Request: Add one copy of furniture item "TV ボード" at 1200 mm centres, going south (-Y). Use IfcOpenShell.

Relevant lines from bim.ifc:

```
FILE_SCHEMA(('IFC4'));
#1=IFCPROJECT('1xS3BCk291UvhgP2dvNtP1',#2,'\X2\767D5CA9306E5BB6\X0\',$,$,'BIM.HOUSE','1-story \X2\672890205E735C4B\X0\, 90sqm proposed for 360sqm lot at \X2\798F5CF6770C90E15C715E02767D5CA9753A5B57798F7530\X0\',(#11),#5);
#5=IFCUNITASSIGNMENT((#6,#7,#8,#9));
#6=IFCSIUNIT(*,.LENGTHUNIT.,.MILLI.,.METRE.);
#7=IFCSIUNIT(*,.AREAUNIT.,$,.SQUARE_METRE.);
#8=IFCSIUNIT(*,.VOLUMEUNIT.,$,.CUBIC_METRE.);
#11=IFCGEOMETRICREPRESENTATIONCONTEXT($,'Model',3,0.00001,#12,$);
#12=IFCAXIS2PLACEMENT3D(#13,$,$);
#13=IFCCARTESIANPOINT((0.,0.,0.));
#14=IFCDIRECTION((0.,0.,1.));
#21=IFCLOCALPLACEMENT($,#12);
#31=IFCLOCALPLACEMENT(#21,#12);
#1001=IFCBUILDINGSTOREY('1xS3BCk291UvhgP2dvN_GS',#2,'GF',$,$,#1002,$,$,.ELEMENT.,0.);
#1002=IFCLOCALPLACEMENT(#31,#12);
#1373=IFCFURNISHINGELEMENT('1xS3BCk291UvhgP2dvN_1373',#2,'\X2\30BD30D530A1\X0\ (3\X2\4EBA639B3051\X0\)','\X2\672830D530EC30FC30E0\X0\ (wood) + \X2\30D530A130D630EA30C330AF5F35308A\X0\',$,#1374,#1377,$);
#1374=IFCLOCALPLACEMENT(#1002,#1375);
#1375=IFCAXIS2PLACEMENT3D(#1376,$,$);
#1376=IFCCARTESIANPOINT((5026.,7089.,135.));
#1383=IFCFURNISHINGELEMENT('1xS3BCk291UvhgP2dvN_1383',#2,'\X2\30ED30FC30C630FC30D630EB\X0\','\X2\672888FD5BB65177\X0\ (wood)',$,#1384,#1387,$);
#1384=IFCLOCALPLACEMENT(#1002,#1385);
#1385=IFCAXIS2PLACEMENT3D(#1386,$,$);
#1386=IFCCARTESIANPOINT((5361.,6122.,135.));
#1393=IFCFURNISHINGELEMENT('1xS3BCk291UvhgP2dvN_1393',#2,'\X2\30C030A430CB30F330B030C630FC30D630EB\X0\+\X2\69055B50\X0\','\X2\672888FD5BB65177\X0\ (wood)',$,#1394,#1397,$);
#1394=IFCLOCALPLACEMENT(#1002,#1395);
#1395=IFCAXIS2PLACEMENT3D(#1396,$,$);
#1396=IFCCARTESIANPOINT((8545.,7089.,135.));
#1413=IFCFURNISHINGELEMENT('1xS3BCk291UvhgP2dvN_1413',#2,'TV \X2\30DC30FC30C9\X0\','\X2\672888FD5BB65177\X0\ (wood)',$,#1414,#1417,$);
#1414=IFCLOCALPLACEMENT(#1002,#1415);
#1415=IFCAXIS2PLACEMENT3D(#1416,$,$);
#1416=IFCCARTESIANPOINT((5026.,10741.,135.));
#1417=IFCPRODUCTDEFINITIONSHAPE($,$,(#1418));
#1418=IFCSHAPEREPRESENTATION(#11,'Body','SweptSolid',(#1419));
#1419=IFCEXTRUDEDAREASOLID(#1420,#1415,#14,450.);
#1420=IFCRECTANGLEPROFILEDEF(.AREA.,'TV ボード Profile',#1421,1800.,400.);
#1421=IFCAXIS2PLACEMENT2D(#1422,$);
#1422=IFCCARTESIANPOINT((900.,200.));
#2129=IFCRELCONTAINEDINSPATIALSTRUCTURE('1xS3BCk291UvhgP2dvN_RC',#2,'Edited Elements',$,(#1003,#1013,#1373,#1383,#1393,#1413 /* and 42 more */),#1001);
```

```python
import numpy as np
import ifcopenshell
import ifcopenshell.api.geometry
import ifcopenshell.api.root
import ifcopenshell.util.element
import ifcopenshell.util.placement
import ifcopenshell.util.unit

model = ifcopenshell.open("bim.ifc")
unit_scale = ifcopenshell.util.unit.calculate_unit_scale(model)


def reuse_history(source, copy):
    """copy_class also copies each property set's owner history, people and application; keep the originals."""
    for rel in copy.IsDefinedBy:
        if rel.is_a("IfcRelDefinesByProperties") and (history := rel.RelatingPropertyDefinition.OwnerHistory):
            rel.RelatingPropertyDefinition.OwnerHistory = source.OwnerHistory
            ifcopenshell.util.element.remove_deep2(model, history)


source = model.by_id(1413)
base = ifcopenshell.util.placement.get_local_placement(source.ObjectPlacement)
step = np.array([0.0, -1.0, 0.0]) * 1.2 / unit_scale

for i in range(1, 2):
    copy = ifcopenshell.api.root.copy_class(model, product=source)
    copy.Representation = ifcopenshell.util.element.copy_deep(
        model, source.Representation, exclude=["IfcGeometricRepresentationContext", "IfcRepresentationMap"]
    )
    reuse_history(source, copy)
    matrix = base.copy()
    matrix[:3, 3] += i * step
    print("added at", matrix[:3, 3].round(3) + 0.0)
    ifcopenshell.api.geometry.edit_object_placement(model, product=copy, matrix=matrix, is_si=False)

model.write("bim_updated.ifc")
```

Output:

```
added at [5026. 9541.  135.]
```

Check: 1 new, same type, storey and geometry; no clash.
